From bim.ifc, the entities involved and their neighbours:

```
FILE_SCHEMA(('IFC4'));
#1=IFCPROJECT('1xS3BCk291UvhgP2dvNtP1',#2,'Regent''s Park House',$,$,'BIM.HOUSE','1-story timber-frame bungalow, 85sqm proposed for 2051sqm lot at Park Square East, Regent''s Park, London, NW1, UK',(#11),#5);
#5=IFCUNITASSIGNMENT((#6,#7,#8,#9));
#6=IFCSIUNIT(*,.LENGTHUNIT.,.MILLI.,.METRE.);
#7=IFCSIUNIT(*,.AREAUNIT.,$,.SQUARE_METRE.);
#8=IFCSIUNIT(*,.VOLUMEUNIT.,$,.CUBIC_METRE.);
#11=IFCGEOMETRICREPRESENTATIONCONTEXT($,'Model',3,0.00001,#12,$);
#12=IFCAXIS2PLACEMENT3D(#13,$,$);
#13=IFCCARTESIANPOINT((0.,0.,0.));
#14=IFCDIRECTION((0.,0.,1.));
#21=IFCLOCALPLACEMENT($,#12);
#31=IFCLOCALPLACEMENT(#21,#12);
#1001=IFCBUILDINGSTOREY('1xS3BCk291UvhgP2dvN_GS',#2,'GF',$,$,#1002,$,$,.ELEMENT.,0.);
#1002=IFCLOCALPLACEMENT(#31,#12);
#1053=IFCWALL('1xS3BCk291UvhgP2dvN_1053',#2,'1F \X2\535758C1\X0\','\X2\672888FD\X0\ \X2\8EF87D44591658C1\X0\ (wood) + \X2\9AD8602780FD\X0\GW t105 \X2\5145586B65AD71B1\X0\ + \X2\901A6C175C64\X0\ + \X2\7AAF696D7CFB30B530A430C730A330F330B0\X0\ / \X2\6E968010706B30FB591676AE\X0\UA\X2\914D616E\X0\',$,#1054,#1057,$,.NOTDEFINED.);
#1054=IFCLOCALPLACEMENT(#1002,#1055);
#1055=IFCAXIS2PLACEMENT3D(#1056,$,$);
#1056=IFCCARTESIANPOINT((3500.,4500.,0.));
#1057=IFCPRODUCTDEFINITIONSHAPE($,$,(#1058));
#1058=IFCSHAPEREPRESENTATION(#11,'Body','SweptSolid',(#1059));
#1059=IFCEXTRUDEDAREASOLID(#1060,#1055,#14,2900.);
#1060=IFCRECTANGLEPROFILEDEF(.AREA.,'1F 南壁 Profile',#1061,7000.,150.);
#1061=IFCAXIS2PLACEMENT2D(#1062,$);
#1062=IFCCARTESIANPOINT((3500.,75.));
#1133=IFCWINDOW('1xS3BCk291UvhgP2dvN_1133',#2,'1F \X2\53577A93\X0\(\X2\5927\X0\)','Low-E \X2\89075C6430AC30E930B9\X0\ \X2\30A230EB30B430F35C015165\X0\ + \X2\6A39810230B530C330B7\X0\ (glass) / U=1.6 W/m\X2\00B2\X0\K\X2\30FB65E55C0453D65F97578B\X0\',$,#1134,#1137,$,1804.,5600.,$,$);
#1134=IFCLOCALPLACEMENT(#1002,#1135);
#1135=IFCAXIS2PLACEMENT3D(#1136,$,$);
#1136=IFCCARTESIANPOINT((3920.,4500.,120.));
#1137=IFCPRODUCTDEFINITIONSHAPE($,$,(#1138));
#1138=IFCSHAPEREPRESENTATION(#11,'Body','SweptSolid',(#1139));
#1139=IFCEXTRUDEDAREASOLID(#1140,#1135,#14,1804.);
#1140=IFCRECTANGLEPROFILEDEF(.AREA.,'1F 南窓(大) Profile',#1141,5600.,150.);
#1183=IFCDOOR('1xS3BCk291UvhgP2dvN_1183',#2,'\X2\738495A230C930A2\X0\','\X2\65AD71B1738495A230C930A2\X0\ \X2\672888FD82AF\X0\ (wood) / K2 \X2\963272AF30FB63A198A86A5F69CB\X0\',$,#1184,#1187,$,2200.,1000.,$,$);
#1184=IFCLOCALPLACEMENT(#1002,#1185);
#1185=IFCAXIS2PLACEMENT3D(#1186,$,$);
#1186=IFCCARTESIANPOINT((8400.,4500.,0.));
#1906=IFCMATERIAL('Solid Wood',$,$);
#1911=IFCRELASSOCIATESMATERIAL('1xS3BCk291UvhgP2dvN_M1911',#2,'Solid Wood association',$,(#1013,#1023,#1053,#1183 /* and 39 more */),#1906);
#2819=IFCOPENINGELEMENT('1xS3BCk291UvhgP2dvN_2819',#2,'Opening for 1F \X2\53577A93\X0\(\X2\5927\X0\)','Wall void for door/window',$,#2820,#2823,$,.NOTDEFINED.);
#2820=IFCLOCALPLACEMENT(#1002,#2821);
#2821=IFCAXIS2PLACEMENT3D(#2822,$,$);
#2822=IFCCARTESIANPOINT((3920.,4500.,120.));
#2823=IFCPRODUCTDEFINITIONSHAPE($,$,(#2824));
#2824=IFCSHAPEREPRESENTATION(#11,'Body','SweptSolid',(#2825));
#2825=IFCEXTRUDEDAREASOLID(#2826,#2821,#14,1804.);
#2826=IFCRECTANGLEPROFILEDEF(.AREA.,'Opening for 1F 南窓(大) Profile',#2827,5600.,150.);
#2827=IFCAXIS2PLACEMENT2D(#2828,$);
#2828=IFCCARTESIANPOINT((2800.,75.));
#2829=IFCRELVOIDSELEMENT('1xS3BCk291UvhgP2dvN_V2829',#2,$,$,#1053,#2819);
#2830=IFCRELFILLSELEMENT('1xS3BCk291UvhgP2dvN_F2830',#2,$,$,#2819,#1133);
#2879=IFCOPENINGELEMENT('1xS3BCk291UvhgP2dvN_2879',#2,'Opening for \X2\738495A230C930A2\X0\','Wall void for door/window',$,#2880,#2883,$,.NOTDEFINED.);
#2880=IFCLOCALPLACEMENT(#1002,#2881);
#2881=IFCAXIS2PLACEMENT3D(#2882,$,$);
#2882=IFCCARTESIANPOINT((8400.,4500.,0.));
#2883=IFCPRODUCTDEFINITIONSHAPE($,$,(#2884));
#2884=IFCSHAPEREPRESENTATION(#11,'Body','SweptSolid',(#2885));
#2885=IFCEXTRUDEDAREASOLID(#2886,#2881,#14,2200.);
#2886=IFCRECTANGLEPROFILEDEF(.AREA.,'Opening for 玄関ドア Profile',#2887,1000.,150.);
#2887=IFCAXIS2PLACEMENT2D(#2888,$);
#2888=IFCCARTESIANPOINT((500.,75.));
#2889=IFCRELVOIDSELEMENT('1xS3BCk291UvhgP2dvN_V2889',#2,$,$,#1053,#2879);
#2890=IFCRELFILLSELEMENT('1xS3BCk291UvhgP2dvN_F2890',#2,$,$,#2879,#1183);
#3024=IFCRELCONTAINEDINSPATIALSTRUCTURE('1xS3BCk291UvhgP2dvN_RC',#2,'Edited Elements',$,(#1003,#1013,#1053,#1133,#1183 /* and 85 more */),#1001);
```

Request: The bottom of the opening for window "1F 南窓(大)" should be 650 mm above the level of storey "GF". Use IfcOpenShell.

```python
import numpy as np
import ifcopenshell
import ifcopenshell.api.geometry
import ifcopenshell.geom
import ifcopenshell.util.element
import ifcopenshell.util.placement
import ifcopenshell.util.shape
import ifcopenshell.util.unit

model = ifcopenshell.open("bim.ifc")
unit_scale = ifcopenshell.util.unit.calculate_unit_scale(model)

window = model.by_guid("1xS3BCk291UvhgP2dvN_1133")
opening = window.FillsVoids[0].RelatingOpeningElement
storey = ifcopenshell.util.element.get_container(window, ifc_class="IfcBuildingStorey")
level = ifcopenshell.util.placement.get_local_placement(storey.ObjectPlacement)[2, 3]

# The opening's origin need not be at the sill, so measure its lowest point.
shape = ifcopenshell.geom.create_shape(ifcopenshell.geom.settings(), opening)
bottom = ifcopenshell.util.shape.get_shape_bottom_elevation(shape, shape.geometry) / unit_scale
dz = level + 0.65 / unit_scale - bottom

shift = np.array([0.0, 0.0, dz])
# The window is not placed relative to its opening, so move both.
for product in (opening, window):
    matrix = ifcopenshell.util.placement.get_local_placement(product.ObjectPlacement)
    matrix[:3, 3] += shift
    ifcopenshell.api.geometry.edit_object_placement(model, product=product, matrix=matrix, is_si=False)

print(f"moved by {dz * unit_scale:+.3f} m")

model.write("bim_edited.ifc")
```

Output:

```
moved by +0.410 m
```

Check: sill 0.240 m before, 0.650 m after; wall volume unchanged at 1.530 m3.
